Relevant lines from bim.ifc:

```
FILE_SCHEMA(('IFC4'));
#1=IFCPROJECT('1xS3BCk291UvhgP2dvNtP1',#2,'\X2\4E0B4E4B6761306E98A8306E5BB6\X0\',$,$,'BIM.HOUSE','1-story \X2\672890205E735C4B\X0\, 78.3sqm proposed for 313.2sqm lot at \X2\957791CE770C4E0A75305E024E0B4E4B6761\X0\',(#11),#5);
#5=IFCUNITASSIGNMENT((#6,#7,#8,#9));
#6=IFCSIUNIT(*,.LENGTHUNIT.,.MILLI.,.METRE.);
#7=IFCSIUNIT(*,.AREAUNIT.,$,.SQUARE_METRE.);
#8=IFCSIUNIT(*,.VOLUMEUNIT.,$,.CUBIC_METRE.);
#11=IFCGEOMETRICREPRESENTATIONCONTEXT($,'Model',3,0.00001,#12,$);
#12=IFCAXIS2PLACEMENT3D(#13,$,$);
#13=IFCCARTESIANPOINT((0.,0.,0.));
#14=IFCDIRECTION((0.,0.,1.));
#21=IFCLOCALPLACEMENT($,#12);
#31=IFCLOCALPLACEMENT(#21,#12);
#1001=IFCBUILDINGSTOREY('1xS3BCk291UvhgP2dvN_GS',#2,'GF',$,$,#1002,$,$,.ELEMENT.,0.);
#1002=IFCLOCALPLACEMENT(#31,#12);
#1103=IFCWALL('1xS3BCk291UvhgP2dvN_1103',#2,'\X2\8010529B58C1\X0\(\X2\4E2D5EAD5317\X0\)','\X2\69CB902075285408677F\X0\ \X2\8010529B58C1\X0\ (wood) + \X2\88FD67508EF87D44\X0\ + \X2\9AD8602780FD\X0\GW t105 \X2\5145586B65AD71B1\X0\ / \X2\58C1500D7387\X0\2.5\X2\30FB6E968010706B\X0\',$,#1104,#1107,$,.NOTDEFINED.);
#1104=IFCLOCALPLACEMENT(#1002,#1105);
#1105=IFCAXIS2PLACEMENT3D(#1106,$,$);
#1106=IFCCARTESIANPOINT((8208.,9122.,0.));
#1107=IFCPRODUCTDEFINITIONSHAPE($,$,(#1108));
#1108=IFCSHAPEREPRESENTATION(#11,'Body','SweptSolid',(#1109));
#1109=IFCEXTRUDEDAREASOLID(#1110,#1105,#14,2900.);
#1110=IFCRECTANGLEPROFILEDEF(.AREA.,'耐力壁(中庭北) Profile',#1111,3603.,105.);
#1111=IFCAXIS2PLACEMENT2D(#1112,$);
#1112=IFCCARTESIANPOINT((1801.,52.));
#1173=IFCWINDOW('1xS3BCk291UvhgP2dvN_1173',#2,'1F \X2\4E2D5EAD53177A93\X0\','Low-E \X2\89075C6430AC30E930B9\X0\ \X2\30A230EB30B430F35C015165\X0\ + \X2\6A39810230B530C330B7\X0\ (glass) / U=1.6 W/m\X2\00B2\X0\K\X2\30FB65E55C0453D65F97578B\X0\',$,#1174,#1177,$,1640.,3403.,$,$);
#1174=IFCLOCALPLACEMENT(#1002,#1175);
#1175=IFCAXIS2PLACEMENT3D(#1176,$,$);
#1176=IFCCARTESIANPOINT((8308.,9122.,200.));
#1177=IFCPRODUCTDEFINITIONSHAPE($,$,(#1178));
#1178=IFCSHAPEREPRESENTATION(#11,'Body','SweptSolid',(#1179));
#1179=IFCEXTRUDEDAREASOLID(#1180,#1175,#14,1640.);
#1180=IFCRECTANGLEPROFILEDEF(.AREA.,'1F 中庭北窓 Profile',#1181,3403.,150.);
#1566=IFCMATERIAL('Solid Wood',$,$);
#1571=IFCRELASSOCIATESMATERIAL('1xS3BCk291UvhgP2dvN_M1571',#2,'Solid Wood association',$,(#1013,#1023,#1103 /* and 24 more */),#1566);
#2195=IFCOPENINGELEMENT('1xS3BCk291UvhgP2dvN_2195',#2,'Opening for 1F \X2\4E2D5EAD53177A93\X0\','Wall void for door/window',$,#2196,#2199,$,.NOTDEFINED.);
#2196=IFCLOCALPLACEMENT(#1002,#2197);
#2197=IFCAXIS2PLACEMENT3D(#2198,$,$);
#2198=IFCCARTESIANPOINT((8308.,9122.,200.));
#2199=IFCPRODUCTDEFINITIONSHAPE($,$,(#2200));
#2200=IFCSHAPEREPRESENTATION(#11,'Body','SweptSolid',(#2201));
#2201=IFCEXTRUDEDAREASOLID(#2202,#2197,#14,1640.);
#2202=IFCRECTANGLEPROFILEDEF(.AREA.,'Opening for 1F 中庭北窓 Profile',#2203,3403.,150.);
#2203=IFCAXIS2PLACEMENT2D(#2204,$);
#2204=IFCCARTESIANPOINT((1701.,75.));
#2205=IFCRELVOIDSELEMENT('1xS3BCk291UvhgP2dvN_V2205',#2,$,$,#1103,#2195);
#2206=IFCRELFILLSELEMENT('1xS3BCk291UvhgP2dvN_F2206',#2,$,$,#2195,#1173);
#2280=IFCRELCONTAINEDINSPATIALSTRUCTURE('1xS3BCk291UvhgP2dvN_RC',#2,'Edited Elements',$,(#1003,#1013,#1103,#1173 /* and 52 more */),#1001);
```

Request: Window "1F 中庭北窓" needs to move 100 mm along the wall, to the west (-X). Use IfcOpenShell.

```python
import ifcopenshell
import ifcopenshell.api.geometry
import ifcopenshell.util.placement

model = ifcopenshell.open("bim.ifc")

window = model.by_guid("1xS3BCk291UvhgP2dvN_1173")
opening = window.FillsVoids[0].RelatingOpeningElement
wall = opening.VoidsElements[0].RelatingBuildingElement

wall_matrix = ifcopenshell.util.placement.get_local_placement(wall.ObjectPlacement)
shift = wall_matrix[:3, 0] * -100.0
before = ifcopenshell.util.placement.get_local_placement(window.ObjectPlacement)[:3, 3].copy()

# The window is not placed relative to its opening, so move both.
for product in (opening, window):
    matrix = ifcopenshell.util.placement.get_local_placement(product.ObjectPlacement)
    matrix[:3, 3] += shift
    ifcopenshell.api.geometry.edit_object_placement(model, product=product, matrix=matrix, is_si=False)

after = ifcopenshell.util.placement.get_local_placement(window.ObjectPlacement)[:3, 3]
print("window moved by", (after - before).round(3) + 0.0)

model.write("bim_v2.ifc")
```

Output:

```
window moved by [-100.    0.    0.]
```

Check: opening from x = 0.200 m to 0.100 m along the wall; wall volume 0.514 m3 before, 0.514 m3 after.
